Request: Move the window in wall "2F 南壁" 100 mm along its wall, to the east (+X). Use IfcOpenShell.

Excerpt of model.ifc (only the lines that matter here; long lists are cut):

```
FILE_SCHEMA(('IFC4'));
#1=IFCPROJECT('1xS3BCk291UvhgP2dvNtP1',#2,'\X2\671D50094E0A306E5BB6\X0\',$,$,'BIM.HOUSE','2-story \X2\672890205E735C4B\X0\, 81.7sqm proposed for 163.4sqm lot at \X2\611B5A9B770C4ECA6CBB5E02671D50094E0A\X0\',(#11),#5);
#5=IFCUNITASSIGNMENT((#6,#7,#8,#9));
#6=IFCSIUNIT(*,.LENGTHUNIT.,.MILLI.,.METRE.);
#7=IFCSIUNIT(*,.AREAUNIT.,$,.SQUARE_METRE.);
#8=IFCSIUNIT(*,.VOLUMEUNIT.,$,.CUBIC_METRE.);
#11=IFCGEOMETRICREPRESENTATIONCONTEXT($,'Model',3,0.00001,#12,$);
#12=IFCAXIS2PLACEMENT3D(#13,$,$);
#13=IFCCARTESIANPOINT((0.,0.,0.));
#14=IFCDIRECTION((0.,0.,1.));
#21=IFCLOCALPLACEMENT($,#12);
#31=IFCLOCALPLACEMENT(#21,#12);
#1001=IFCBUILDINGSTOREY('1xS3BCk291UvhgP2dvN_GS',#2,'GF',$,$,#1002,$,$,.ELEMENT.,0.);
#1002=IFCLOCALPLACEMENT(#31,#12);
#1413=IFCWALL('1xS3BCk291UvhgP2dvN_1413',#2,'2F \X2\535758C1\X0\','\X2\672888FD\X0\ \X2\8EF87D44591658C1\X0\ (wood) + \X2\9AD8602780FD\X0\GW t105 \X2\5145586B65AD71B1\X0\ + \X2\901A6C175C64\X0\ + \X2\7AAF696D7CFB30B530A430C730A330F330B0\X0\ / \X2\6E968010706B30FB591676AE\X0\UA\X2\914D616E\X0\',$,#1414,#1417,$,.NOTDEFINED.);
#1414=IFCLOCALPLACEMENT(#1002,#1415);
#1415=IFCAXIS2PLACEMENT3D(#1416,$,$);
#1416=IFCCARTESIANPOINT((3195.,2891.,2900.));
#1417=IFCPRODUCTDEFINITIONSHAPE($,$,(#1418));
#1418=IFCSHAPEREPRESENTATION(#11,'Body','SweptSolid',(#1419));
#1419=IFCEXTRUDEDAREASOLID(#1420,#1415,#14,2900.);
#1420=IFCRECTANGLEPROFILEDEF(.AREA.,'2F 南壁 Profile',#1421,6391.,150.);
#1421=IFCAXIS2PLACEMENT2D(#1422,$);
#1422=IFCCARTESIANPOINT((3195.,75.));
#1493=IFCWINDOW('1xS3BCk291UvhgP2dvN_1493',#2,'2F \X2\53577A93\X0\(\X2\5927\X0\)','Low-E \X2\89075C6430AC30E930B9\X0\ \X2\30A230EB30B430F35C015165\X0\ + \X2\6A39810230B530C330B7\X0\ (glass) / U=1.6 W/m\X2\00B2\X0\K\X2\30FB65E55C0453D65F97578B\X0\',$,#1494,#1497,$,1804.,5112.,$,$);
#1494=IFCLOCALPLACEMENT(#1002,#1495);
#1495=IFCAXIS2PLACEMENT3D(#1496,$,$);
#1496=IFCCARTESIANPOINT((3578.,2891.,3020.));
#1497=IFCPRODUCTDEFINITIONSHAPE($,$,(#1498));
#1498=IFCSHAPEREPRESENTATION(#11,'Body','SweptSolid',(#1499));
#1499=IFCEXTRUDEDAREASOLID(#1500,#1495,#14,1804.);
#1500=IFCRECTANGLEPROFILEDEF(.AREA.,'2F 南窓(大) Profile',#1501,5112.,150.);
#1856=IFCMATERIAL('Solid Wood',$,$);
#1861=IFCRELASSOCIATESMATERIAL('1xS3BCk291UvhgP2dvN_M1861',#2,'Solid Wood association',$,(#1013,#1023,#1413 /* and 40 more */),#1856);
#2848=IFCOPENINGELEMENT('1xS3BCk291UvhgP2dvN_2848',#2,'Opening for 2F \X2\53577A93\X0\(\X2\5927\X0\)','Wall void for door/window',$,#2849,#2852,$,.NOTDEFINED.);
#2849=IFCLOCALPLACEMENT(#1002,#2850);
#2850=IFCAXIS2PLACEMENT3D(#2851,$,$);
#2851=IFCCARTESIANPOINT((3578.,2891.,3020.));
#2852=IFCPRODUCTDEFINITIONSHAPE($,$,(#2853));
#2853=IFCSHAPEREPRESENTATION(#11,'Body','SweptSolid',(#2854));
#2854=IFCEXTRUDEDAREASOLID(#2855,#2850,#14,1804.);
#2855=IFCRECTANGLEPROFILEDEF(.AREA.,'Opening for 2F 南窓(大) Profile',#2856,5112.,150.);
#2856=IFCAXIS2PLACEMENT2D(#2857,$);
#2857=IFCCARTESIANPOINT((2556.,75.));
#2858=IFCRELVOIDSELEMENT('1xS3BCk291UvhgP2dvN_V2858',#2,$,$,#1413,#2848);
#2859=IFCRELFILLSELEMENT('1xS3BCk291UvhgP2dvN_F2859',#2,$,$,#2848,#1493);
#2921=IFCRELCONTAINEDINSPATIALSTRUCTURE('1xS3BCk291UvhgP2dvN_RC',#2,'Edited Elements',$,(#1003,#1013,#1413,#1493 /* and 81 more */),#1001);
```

```python
import ifcopenshell
import ifcopenshell.api.geometry
import ifcopenshell.util.placement
import ifcopenshell.util.unit

model = ifcopenshell.open("model.ifc")
unit_scale = ifcopenshell.util.unit.calculate_unit_scale(model)

window = model.by_guid("1xS3BCk291UvhgP2dvN_1493")
opening = window.FillsVoids[0].RelatingOpeningElement
wall = opening.VoidsElements[0].RelatingBuildingElement

wall_matrix = ifcopenshell.util.placement.get_local_placement(wall.ObjectPlacement)
shift = wall_matrix[:3, 0] * 0.1 / unit_scale
before = ifcopenshell.util.placement.get_local_placement(window.ObjectPlacement)[:3, 3].copy()

# The window is not placed relative to its opening, so move both.
for product in (opening, window):
    matrix = ifcopenshell.util.placement.get_local_placement(product.ObjectPlacement)
    matrix[:3, 3] += shift
    ifcopenshell.api.geometry.edit_object_placement(model, product=product, matrix=matrix, is_si=False)

after = ifcopenshell.util.placement.get_local_placement(window.ObjectPlacement)[:3, 3]
print("window moved by", (after - before).round(3) + 0.0)

model.write("model-out.ifc")
```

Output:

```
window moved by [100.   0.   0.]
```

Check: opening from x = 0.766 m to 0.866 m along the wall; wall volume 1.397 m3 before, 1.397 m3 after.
